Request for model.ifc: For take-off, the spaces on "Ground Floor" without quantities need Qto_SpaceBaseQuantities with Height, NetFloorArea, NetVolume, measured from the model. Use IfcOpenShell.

First a look at what the model holds.

```python
import ifcopenshell
import ifcopenshell.util.element
import ifcopenshell.util.unit

model = ifcopenshell.open("model.ifc")
print(model.schema)
for unit_type in ("LENGTHUNIT", "AREAUNIT", "VOLUMEUNIT"):
    print(unit_type, ifcopenshell.util.unit.calculate_unit_scale(model, unit_type))
storey = next(s for s in model.by_type("IfcBuildingStorey") if s.Name == "Ground Floor")
spaces = [e for e in ifcopenshell.util.element.get_decomposition(storey) if e.is_a("IfcSpace")]
for e in sorted(spaces, key=lambda e: e.id()):
    print(e.id(), e.is_a(), e.Name, list(ifcopenshell.util.element.get_psets(e, qtos_only=True)), sep=" | ")
```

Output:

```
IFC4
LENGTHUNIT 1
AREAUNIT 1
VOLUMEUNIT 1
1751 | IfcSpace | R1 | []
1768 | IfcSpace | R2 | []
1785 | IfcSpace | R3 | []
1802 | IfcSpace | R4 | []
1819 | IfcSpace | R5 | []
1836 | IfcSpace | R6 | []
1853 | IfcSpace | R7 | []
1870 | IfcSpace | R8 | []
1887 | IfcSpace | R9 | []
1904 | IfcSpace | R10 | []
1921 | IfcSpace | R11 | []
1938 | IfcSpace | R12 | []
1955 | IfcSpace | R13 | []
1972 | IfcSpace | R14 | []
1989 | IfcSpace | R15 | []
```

```python
import ifcopenshell
import ifcopenshell.api.pset
import ifcopenshell.geom
import ifcopenshell.util.element
import ifcopenshell.util.shape
import ifcopenshell.util.unit

model = ifcopenshell.open("model.ifc")
unit_scale = ifcopenshell.util.unit.calculate_unit_scale(model)
area_scale = ifcopenshell.util.unit.calculate_unit_scale(model, "AREAUNIT")
volume_scale = ifcopenshell.util.unit.calculate_unit_scale(model, "VOLUMEUNIT")
settings = ifcopenshell.geom.settings()

storey = next(s for s in model.by_type("IfcBuildingStorey") if s.Name == "Ground Floor")
spaces = [e for e in ifcopenshell.util.element.get_decomposition(storey) if e.is_a("IfcSpace")]

for e in sorted(spaces, key=lambda e: e.id()):
    if ifcopenshell.util.element.get_psets(e, qtos_only=True, should_inherit=False):
        continue
    # Geometry comes back in metres, in the element's own axes.
    shape = ifcopenshell.geom.create_shape(settings, e)
    values = {
        "Height": ifcopenshell.util.shape.get_z(shape.geometry) / unit_scale,
        "NetFloorArea": ifcopenshell.util.shape.get_footprint_area(shape.geometry) / area_scale,
        "NetVolume": ifcopenshell.util.shape.get_volume(shape.geometry) / volume_scale,
    }
    qto = ifcopenshell.api.pset.add_qto(model, product=e, name="Qto_SpaceBaseQuantities")
    ifcopenshell.api.pset.edit_qto(model, qto=qto, properties=values)
    print(e.id(), {k: round(v, 3) for k, v in values.items()})

model.write("model_rev.ifc")
```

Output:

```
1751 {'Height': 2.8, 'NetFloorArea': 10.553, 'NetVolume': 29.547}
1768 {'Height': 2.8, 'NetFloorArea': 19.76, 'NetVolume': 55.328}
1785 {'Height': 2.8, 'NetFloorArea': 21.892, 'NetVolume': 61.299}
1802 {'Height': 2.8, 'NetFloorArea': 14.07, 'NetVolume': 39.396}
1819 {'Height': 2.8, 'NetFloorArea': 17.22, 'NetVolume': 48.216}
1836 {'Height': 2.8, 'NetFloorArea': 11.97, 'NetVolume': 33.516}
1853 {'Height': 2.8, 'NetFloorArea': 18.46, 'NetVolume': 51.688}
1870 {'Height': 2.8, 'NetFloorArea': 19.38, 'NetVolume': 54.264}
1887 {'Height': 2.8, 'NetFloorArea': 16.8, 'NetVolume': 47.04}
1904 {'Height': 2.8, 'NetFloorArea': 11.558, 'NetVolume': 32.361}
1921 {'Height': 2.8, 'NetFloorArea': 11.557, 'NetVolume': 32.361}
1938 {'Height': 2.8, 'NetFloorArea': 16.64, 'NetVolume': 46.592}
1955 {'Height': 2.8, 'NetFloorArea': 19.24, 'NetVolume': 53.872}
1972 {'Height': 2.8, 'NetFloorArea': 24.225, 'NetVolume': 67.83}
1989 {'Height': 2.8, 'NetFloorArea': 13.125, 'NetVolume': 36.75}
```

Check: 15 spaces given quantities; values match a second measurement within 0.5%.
